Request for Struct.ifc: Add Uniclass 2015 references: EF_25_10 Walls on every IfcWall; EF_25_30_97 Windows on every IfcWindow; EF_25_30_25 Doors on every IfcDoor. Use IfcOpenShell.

First a look at what the model holds.

```python
import ifcopenshell

model = ifcopenshell.open("Struct.ifc")
print(model.schema)
print("classifications:", [c.Name for c in model.by_type("IfcClassification")])
for ifc_class in ("IfcDoor", "IfcRoof", "IfcStair", "IfcWall", "IfcWindow"):
    print(ifc_class, len(model.by_type(ifc_class)))
```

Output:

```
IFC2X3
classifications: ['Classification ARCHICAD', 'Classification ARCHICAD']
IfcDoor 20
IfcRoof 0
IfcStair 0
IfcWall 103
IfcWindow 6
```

```python
import ifcopenshell
import ifcopenshell.api.classification

model = ifcopenshell.open("Struct.ifc")

# IFC2X3 requires Source and Edition and has no link from the project to the system.
system = model.create_entity("IfcClassification", Source="NBS", Edition="2015", Name="Uniclass 2015")

codes = {
    "IfcWall": ("EF_25_10", "Walls"),
    "IfcWindow": ("EF_25_30_97", "Windows"),
    "IfcDoor": ("EF_25_30_25", "Doors"),
}
for ifc_class, (code, name) in codes.items():
    products = model.by_type(ifc_class)
    ifcopenshell.api.classification.add_reference(
        model, products=products, classification=system, identification=code, name=name
    )
    print(code, len(products))

model.write("Struct-out.ifc")
```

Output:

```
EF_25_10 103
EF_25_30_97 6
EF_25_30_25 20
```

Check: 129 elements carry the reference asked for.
